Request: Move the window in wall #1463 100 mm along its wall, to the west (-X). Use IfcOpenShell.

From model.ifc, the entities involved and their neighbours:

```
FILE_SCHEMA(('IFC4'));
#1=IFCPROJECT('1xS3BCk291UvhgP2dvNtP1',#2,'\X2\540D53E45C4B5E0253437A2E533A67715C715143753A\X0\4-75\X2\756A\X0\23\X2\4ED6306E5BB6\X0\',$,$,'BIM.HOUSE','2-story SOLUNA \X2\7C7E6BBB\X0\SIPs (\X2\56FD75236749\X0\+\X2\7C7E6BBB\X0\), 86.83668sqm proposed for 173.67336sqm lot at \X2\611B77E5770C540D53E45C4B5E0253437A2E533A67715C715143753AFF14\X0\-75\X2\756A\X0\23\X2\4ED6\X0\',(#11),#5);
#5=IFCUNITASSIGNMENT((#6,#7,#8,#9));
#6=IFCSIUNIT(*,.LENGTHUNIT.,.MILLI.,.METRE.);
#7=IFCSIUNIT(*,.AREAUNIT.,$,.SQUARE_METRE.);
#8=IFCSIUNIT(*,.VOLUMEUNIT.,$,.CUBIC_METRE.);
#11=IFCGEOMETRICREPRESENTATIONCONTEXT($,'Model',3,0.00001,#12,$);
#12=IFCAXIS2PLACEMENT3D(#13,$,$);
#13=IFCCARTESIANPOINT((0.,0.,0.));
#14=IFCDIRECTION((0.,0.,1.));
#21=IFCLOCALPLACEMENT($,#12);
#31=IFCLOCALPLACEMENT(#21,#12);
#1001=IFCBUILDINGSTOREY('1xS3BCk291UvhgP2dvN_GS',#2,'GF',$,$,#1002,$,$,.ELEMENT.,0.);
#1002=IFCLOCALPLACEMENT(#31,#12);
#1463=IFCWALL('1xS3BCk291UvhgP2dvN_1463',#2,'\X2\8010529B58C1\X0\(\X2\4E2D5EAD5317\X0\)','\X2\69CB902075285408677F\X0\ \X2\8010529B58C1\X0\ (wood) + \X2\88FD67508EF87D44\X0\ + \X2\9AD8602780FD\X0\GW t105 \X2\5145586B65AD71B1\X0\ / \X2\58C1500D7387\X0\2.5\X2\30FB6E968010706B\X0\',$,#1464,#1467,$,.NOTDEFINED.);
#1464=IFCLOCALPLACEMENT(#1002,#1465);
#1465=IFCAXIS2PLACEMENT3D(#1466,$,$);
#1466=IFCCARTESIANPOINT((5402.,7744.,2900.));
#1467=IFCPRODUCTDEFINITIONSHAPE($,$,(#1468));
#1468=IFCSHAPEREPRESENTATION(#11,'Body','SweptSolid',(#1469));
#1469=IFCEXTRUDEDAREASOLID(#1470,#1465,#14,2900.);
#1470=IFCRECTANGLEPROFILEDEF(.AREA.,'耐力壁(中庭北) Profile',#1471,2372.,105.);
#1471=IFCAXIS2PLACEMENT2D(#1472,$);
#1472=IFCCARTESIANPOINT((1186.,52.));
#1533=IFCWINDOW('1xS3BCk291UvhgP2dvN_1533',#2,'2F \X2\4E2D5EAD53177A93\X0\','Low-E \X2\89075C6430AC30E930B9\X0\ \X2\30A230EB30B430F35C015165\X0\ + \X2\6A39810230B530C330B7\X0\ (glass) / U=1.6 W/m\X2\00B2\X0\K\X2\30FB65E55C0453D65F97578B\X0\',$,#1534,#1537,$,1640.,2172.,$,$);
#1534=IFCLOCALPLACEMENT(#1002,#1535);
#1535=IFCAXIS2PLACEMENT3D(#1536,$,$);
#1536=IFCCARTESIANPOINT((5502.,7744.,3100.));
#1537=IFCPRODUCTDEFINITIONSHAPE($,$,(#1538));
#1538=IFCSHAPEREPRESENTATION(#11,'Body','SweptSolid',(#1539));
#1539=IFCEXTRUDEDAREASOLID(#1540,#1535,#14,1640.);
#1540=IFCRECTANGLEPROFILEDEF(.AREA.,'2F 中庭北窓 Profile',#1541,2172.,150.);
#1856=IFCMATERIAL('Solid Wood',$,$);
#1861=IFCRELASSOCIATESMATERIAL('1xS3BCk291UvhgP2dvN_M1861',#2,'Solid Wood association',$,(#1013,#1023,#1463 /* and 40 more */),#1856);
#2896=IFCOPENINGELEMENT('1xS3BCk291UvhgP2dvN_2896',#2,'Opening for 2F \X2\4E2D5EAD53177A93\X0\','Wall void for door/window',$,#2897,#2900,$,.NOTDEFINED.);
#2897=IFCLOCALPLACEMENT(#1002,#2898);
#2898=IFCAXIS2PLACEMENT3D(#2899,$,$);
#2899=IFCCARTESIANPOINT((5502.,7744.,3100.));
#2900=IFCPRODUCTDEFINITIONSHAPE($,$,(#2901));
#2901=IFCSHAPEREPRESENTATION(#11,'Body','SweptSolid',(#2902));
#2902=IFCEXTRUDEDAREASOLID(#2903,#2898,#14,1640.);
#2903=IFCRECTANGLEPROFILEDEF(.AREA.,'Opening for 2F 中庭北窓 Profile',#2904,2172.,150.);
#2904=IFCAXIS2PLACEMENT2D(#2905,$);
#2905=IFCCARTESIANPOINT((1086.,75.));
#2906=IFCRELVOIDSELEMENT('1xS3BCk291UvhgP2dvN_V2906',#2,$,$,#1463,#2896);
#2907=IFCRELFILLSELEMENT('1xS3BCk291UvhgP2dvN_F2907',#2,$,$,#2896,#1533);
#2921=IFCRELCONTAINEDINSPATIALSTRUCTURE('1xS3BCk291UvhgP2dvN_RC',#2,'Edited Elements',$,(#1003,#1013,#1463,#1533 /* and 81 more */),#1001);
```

```python
import ifcopenshell
import ifcopenshell.api.geometry
import ifcopenshell.util.placement
import ifcopenshell.util.unit

model = ifcopenshell.open("model.ifc")
unit_scale = ifcopenshell.util.unit.calculate_unit_scale(model)

window = model.by_guid("1xS3BCk291UvhgP2dvN_1533")
opening = window.FillsVoids[0].RelatingOpeningElement
wall = opening.VoidsElements[0].RelatingBuildingElement

wall_matrix = ifcopenshell.util.placement.get_local_placement(wall.ObjectPlacement)
shift = wall_matrix[:3, 0] * -0.1 / unit_scale
before = ifcopenshell.util.placement.get_local_placement(window.ObjectPlacement)[:3, 3].copy()

# The window is not placed relative to its opening, so move both.
for product in (opening, window):
    matrix = ifcopenshell.util.placement.get_local_placement(product.ObjectPlacement)
    matrix[:3, 3] += shift
    ifcopenshell.api.geometry.edit_object_placement(model, product=product, matrix=matrix, is_si=False)

after = ifcopenshell.util.placement.get_local_placement(window.ObjectPlacement)[:3, 3]
print("window moved by", (after - before).round(3) + 0.0)

model.write("model_edited.ifc")
```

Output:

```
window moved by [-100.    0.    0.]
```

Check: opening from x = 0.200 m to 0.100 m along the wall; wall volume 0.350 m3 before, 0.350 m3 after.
